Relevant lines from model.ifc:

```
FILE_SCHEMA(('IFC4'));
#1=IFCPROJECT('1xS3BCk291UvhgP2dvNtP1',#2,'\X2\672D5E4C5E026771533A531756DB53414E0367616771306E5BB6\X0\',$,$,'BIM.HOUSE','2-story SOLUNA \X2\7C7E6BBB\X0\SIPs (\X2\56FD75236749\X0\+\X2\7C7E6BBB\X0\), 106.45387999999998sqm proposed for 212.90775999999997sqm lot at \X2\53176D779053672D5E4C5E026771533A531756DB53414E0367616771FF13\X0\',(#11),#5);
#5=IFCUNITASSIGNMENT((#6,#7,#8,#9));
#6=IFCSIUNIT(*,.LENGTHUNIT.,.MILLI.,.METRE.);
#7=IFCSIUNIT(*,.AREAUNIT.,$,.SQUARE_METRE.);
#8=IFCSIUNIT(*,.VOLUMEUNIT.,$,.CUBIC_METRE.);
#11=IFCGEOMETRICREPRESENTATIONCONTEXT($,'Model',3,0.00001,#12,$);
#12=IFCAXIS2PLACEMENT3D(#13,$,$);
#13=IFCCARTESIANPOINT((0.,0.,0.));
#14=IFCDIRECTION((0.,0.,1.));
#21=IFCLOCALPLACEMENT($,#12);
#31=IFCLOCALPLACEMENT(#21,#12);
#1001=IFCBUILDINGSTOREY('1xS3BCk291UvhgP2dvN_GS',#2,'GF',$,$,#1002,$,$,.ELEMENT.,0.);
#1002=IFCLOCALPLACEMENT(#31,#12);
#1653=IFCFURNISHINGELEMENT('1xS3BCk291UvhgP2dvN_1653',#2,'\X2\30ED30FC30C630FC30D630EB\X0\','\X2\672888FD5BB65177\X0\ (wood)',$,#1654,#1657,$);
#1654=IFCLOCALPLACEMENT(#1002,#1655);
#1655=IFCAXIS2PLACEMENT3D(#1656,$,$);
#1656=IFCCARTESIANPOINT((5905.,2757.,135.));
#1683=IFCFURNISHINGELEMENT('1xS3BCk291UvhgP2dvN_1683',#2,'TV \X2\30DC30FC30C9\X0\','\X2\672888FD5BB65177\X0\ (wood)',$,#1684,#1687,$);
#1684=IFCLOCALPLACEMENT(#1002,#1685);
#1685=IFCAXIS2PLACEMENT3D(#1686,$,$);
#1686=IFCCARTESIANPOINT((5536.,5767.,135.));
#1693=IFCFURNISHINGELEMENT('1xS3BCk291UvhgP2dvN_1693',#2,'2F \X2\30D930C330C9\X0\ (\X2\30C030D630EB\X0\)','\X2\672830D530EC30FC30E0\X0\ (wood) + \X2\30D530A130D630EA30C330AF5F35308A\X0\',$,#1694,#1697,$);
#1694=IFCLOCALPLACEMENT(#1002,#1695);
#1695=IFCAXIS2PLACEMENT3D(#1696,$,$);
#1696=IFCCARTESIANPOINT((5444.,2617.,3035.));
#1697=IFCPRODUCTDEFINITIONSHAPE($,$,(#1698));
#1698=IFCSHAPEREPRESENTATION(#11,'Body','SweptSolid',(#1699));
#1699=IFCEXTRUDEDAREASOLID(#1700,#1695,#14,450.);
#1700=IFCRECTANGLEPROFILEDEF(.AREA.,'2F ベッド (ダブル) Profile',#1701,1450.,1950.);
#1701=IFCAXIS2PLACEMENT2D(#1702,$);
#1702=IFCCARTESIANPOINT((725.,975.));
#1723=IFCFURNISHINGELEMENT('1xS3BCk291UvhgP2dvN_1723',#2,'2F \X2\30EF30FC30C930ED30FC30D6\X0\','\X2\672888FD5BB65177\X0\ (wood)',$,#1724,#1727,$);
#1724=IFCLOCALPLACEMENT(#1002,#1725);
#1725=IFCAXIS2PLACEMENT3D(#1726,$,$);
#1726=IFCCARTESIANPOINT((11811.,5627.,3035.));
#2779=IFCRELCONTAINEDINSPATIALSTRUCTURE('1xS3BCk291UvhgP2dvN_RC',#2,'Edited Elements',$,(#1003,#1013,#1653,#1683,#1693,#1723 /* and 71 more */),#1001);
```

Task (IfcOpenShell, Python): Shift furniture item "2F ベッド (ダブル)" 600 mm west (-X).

```python
import ifcopenshell
import ifcopenshell.api.geometry
import ifcopenshell.util.placement
import ifcopenshell.util.unit

model = ifcopenshell.open("model.ifc")
unit_scale = ifcopenshell.util.unit.calculate_unit_scale(model)

item = model.by_guid("1xS3BCk291UvhgP2dvN_1693")
matrix = ifcopenshell.util.placement.get_local_placement(item.ObjectPlacement)
matrix[0, 3] -= 0.6 / unit_scale
ifcopenshell.api.geometry.edit_object_placement(model, product=item, matrix=matrix, is_si=False)

print(ifcopenshell.util.placement.get_local_placement(item.ObjectPlacement).round(3) + 0.0)

model.write("model_updated.ifc")
```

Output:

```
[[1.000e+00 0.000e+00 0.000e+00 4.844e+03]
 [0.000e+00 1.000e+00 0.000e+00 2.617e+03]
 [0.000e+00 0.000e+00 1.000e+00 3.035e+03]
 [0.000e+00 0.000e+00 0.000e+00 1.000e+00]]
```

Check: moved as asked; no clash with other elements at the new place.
